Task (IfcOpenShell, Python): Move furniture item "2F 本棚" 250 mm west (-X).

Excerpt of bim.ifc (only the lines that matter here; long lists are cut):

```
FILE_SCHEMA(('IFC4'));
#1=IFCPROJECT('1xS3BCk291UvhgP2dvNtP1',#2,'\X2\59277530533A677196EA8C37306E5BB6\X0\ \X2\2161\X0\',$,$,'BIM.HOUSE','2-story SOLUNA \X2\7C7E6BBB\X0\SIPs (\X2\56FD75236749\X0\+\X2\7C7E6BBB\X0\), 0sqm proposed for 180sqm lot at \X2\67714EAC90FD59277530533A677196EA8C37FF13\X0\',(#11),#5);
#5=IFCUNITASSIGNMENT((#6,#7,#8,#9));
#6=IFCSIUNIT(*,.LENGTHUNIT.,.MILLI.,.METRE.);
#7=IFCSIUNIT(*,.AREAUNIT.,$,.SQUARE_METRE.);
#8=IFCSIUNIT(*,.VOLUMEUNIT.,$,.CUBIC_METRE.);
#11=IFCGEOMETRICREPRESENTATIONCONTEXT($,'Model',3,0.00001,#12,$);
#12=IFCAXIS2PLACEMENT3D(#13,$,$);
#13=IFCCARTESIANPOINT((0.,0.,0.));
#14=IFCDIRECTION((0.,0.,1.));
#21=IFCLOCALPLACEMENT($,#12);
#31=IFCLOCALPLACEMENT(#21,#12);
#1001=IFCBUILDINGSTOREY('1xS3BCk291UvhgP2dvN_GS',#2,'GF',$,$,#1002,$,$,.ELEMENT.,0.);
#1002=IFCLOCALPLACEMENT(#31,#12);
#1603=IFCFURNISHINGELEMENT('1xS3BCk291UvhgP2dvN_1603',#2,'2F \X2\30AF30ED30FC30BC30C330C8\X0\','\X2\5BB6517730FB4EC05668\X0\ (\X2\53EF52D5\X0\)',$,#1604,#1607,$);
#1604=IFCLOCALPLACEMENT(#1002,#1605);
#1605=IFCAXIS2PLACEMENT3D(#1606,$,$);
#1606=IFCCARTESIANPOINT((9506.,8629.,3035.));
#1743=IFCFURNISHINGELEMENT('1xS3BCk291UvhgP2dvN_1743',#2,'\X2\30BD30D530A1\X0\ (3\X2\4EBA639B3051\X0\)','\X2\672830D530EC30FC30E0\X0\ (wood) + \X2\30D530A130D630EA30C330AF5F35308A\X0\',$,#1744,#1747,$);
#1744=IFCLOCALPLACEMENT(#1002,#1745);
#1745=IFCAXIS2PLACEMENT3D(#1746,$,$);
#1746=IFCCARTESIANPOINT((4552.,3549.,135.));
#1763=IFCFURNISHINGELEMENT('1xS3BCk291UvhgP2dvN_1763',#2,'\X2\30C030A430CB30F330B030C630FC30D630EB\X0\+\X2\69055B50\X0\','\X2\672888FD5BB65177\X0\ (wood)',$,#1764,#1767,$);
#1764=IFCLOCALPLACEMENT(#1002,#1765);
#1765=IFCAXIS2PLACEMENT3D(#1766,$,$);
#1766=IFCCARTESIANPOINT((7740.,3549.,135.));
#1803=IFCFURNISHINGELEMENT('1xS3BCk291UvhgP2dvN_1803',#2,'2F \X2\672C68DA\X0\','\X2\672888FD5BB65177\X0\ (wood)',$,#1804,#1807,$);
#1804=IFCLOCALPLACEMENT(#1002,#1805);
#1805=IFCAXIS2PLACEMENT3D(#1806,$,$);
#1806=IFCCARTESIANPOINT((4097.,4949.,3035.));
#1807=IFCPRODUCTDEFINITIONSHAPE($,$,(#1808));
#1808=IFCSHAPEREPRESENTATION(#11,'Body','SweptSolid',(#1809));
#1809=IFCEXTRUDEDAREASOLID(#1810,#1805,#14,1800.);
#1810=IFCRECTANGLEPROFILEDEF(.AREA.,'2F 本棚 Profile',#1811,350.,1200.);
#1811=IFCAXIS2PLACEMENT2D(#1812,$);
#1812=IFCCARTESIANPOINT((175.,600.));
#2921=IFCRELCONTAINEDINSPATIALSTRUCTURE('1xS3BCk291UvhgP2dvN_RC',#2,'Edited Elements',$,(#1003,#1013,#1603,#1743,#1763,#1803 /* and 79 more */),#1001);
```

```python
import ifcopenshell
import ifcopenshell.api.geometry
import ifcopenshell.util.placement
import ifcopenshell.util.unit

model = ifcopenshell.open("bim.ifc")
unit_scale = ifcopenshell.util.unit.calculate_unit_scale(model)

item = model.by_id(1803)
matrix = ifcopenshell.util.placement.get_local_placement(item.ObjectPlacement)
matrix[0, 3] -= 0.25 / unit_scale
ifcopenshell.api.geometry.edit_object_placement(model, product=item, matrix=matrix, is_si=False)

print(ifcopenshell.util.placement.get_local_placement(item.ObjectPlacement).round(3) + 0.0)

model.write("bim_edited.ifc")
```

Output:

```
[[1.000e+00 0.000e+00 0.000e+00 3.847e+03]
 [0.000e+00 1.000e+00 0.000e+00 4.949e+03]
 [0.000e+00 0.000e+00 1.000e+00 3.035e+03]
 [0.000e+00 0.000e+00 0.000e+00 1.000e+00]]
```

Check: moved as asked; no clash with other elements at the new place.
